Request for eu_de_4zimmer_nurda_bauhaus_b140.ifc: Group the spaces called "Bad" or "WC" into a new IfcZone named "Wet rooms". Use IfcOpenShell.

First a look at what the model holds.

```python
import ifcopenshell

model = ifcopenshell.open("eu_de_4zimmer_nurda_bauhaus_b140.ifc")
print(model.schema)
seen = {}
for space in model.by_type("IfcSpace"):
    seen[space.LongName] = seen.get(space.LongName, 0) + 1
for name, count in sorted(seen.items(), key=str):
    print(count, "x", name)
print("zones:", [z.Name for z in model.by_type("IfcZone")][:20])
```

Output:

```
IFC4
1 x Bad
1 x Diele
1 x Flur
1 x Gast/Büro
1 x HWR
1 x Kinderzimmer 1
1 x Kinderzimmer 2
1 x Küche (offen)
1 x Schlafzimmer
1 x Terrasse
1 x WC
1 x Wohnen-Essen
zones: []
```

```python
import ifcopenshell
import ifcopenshell.api.group
import ifcopenshell.api.root

model = ifcopenshell.open("eu_de_4zimmer_nurda_bauhaus_b140.ifc")

names = {"Bad", "WC"}
spaces = [s for s in model.by_type("IfcSpace") if s.LongName in names]

zone = ifcopenshell.api.root.create_entity(model, ifc_class="IfcZone", name="Wet rooms")
ifcopenshell.api.group.assign_group(model, products=spaces, group=zone)
print(len(spaces), "spaces in", zone.Name)

model.write("eu_de_4zimmer_nurda_bauhaus_b140_v2.ifc")
```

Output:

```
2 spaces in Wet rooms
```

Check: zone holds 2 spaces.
